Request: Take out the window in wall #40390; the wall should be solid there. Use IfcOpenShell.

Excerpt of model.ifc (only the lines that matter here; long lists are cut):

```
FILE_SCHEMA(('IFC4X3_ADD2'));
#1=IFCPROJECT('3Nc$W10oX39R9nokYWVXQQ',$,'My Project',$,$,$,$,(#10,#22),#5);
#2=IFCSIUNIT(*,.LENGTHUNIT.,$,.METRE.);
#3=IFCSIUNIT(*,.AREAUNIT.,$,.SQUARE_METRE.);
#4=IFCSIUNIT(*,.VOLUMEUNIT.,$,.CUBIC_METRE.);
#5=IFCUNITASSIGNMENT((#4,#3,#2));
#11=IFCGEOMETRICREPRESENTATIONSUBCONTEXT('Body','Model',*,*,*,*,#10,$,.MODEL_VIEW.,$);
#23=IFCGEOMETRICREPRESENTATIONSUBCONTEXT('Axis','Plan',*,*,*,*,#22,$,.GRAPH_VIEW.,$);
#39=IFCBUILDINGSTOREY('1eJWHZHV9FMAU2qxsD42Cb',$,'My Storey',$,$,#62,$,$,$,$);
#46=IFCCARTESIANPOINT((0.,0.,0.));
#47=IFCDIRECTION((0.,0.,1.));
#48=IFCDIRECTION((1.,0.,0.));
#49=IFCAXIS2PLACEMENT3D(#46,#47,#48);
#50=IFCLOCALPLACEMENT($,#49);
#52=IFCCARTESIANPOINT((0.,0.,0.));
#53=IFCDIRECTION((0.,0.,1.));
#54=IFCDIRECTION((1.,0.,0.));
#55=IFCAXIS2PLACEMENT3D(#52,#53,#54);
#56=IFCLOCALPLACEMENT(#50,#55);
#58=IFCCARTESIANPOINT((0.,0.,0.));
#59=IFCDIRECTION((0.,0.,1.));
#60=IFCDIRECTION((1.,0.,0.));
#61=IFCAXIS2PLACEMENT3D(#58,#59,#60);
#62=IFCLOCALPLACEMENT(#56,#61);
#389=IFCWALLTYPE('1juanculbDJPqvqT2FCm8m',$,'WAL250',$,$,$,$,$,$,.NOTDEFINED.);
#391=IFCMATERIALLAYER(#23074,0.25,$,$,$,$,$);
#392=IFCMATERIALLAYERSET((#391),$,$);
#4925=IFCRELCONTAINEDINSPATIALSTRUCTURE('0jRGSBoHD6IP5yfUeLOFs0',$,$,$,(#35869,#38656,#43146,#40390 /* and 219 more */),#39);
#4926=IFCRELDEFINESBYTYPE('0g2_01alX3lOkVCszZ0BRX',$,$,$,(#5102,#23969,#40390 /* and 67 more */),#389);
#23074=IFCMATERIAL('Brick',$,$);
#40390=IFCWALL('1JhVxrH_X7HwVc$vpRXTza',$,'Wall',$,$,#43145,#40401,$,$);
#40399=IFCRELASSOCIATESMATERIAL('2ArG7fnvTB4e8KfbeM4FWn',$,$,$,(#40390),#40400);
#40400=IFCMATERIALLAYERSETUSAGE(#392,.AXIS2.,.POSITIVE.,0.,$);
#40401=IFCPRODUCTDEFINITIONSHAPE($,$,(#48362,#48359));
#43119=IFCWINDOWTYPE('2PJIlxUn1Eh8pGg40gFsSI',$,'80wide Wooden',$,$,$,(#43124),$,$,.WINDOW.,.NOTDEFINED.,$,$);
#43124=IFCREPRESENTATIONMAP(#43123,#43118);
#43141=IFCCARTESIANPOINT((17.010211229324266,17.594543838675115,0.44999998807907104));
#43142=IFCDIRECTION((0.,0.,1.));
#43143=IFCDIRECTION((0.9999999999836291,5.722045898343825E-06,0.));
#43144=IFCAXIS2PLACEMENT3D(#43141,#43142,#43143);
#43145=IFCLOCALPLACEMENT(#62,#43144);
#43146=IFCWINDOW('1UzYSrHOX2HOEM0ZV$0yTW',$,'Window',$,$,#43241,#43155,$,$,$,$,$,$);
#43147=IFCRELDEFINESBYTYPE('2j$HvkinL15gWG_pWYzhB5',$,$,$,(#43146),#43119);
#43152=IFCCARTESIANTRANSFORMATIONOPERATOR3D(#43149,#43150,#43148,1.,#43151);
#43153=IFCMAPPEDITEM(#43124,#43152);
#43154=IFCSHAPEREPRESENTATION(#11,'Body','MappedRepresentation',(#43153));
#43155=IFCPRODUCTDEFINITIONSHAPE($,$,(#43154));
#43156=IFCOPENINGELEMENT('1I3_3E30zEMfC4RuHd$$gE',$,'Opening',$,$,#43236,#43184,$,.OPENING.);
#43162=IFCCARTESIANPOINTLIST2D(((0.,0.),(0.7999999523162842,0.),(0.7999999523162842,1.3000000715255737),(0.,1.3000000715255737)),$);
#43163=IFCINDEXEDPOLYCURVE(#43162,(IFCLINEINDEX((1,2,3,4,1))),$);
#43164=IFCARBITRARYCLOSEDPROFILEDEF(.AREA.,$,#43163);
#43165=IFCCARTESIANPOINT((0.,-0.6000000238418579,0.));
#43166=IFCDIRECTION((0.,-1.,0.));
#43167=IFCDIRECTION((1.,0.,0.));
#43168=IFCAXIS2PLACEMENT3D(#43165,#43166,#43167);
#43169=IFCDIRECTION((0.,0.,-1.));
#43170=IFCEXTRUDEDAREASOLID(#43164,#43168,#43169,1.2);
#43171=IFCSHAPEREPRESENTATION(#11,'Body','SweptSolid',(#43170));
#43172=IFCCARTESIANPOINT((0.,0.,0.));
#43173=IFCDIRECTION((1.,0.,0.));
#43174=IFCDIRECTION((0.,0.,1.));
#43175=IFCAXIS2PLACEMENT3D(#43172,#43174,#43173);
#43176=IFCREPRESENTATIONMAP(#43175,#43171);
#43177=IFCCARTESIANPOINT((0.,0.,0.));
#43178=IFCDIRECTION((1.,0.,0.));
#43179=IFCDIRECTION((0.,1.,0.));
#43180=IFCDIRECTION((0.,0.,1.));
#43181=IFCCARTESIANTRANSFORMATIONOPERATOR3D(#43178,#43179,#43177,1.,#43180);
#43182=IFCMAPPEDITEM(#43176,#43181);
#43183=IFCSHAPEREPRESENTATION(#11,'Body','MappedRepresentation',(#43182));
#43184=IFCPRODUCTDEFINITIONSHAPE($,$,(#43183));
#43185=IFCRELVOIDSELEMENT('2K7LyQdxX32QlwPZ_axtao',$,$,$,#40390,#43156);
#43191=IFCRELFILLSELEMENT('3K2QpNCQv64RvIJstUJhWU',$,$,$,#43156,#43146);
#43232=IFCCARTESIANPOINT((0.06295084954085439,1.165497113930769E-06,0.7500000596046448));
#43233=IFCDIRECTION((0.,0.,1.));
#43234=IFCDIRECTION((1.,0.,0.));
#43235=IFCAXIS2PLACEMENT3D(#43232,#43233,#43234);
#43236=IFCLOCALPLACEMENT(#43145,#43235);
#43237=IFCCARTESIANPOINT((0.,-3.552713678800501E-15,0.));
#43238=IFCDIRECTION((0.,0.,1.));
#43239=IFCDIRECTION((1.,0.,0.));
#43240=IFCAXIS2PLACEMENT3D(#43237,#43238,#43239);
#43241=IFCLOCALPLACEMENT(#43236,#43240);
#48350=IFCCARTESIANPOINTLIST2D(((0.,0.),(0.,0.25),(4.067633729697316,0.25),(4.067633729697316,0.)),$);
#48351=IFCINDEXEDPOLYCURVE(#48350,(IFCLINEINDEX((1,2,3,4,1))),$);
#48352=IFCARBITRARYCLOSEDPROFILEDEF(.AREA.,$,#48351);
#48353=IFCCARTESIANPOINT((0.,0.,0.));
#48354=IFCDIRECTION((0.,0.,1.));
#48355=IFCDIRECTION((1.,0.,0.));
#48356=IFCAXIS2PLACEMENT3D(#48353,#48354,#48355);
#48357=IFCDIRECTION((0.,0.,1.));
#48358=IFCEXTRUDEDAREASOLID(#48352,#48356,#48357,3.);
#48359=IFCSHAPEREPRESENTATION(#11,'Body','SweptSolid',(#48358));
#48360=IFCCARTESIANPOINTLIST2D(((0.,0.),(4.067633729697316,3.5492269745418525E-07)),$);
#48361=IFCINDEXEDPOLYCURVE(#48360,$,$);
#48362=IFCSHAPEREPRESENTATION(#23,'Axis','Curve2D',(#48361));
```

```python
import ifcopenshell
import ifcopenshell.api.feature
import ifcopenshell.api.root
import ifcopenshell.geom
import ifcopenshell.util.shape

model = ifcopenshell.open("model.ifc")
settings = ifcopenshell.geom.settings()


def volume(element):
    """Net volume in cubic metres, openings subtracted."""
    shape = ifcopenshell.geom.create_shape(settings, element)
    return ifcopenshell.util.shape.get_volume(shape.geometry)


window = model.by_id(43146)
opening = window.FillsVoids[0].RelatingOpeningElement
wall = opening.VoidsElements[0].RelatingBuildingElement
before = volume(wall)

ifcopenshell.api.root.remove_product(model, product=window)
ifcopenshell.api.feature.remove_feature(model, feature=opening)

after = volume(wall)

print(f"wall volume {before:.3f} -> {after:.3f} m3")

model.write("model_rev.ifc")
```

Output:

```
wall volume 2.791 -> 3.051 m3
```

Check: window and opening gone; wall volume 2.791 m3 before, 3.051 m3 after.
